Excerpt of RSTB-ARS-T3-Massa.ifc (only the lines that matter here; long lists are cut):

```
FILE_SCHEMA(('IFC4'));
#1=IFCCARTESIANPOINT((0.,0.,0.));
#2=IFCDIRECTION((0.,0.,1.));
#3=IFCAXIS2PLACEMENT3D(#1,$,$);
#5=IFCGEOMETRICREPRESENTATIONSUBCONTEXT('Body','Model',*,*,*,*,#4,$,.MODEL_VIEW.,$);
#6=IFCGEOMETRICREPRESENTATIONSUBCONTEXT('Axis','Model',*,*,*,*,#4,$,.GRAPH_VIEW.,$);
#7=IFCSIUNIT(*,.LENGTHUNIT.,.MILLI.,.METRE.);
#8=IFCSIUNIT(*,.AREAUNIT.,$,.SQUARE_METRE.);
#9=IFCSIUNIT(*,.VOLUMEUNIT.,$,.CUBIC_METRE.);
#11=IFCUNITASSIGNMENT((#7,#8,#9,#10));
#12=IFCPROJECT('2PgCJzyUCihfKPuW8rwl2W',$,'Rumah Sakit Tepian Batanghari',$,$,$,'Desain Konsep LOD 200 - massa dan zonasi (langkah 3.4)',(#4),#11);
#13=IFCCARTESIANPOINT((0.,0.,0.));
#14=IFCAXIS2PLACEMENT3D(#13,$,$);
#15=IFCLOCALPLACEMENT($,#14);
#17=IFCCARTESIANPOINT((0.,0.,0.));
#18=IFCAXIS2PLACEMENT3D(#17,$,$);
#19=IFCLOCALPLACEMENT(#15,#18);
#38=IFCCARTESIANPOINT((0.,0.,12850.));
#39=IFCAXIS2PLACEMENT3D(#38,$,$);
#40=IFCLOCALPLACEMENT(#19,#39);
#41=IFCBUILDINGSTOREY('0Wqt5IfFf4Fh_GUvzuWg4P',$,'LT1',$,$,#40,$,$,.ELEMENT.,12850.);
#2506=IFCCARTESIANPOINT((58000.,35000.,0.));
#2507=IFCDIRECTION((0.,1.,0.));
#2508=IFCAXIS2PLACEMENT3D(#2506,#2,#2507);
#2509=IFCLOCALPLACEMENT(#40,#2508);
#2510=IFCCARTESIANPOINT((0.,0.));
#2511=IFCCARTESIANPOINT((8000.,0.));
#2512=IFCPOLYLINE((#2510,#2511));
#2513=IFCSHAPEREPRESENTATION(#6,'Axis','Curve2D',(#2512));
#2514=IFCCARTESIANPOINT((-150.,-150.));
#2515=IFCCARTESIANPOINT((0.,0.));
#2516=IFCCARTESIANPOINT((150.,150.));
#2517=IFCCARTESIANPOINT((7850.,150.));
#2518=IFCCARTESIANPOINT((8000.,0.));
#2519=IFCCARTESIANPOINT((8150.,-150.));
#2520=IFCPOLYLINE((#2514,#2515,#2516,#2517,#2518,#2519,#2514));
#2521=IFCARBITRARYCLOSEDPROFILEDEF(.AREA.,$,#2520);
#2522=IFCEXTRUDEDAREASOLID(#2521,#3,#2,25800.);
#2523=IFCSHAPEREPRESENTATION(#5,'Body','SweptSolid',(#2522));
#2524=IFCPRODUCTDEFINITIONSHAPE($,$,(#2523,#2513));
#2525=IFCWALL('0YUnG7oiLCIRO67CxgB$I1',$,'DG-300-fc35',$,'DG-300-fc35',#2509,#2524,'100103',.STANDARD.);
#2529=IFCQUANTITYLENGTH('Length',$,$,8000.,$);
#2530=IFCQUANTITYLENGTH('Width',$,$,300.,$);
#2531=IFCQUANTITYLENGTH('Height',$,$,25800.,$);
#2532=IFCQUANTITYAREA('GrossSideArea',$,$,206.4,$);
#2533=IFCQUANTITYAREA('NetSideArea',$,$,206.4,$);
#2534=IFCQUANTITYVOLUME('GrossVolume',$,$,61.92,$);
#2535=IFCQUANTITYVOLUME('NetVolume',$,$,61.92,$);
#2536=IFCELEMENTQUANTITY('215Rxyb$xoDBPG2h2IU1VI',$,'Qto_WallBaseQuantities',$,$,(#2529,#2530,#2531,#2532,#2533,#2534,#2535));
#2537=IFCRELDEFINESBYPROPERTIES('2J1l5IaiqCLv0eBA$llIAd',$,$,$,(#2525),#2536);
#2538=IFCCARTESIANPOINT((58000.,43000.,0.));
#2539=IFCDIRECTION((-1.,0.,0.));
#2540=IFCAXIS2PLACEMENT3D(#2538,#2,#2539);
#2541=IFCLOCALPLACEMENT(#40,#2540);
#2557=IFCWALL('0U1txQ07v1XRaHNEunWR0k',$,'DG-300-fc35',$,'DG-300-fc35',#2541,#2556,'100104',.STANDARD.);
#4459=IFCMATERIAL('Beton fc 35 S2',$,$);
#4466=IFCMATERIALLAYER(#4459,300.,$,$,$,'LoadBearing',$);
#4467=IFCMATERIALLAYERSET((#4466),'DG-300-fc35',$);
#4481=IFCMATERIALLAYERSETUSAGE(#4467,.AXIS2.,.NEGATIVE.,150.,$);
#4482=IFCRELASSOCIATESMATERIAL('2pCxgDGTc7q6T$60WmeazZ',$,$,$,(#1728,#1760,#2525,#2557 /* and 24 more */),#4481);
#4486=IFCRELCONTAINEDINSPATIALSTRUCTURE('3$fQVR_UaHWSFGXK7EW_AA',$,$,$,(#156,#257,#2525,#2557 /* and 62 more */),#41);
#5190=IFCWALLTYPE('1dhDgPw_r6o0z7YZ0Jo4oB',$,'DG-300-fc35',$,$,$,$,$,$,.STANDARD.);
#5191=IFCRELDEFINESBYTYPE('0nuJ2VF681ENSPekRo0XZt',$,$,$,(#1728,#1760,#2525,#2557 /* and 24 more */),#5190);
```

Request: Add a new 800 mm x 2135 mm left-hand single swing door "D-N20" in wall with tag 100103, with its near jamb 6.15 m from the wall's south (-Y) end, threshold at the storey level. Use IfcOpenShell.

```python
import numpy as np
import ifcopenshell
import ifcopenshell.api.feature
import ifcopenshell.api.geometry
import ifcopenshell.api.pset
import ifcopenshell.api.root
import ifcopenshell.api.spatial
import ifcopenshell.geom
import ifcopenshell.util.element
import ifcopenshell.util.placement
import ifcopenshell.util.representation
import ifcopenshell.util.shape
import ifcopenshell.util.unit

model = ifcopenshell.open("RSTB-ARS-T3-Massa.ifc")
unit_scale = ifcopenshell.util.unit.calculate_unit_scale(model)
area_scale = ifcopenshell.util.unit.calculate_unit_scale(model, "AREAUNIT")
volume_scale = ifcopenshell.util.unit.calculate_unit_scale(model, "VOLUMEUNIT")
settings = ifcopenshell.geom.settings()


def volume(element):
    """Net volume in cubic metres, openings subtracted."""
    shape = ifcopenshell.geom.create_shape(settings, element)
    return ifcopenshell.util.shape.get_volume(shape.geometry)


wall = model.by_guid("0YUnG7oiLCIRO67CxgB$I1")
storey = ifcopenshell.util.element.get_container(wall, ifc_class="IfcBuildingStorey")
context = ifcopenshell.util.representation.get_context(model, "Model", "Body", "MODEL_VIEW")
before = volume(wall)

width, height, from_end, sill = 0.8, 2.135, 6.15, 0.0  # metres

# The wall runs along its own X axis, and the end named is its -X end.
wall_shape = ifcopenshell.geom.create_shape(settings, wall)
x, y, z = ifcopenshell.util.shape.get_vertices(wall_shape.geometry).T
start = x.min() + from_end
face, thickness = float(y.min()), float(y.max() - y.min())
wall_matrix = ifcopenshell.util.placement.get_local_placement(wall.ObjectPlacement)
level = ifcopenshell.util.placement.get_local_placement(storey.ObjectPlacement)[2, 3]


def in_wall(x, y):
    """Placement at x, y metres in the wall's axes, at sill height."""
    matrix = wall_matrix.copy()
    matrix[:, 3] = wall_matrix @ np.array([x / unit_scale, y / unit_scale, 0.0, 1.0])
    matrix[2, 3] = level + sill / unit_scale
    return matrix


# Opening: a box that overshoots both wall faces by 50 mm.
opening = ifcopenshell.api.root.create_entity(model, ifc_class="IfcOpeningElement", predefined_type="OPENING")
box = ifcopenshell.api.geometry.add_wall_representation(
    model, context=context, length=width, height=height, thickness=thickness + 0.1
)
ifcopenshell.api.geometry.assign_representation(model, product=opening, representation=box)
ifcopenshell.api.geometry.edit_object_placement(model, product=opening, matrix=in_wall(start, face - 0.05), is_si=False)
ifcopenshell.api.feature.add_feature(model, feature=opening, element=wall)

door = ifcopenshell.api.root.create_entity(model, ifc_class="IfcDoor", name="D-N20", predefined_type="DOOR")
door.OverallWidth, door.OverallHeight = width / unit_scale, height / unit_scale
door.OperationType = "SINGLE_SWING_LEFT"
body = ifcopenshell.api.geometry.add_door_representation(
    model,
    context=context,
    overall_width=door.OverallWidth,
    overall_height=door.OverallHeight,
    operation_type="SINGLE_SWING_LEFT",
    lining_properties={"LiningDepth": thickness / unit_scale, "ThresholdDepth": thickness / unit_scale},
)
ifcopenshell.api.geometry.assign_representation(model, product=door, representation=body)
ifcopenshell.api.spatial.assign_container(model, products=[door], relating_structure=storey)
ifcopenshell.api.feature.add_filling(model, opening=opening, element=door)

# The lining spans the wall, so the door starts at the wall face.
ifcopenshell.api.geometry.edit_object_placement(model, product=door, matrix=in_wall(start, face), is_si=False)

after = volume(wall)

# Update the wall's stored quantities.
qto = model.by_id(ifcopenshell.util.element.get_pset(wall, "Qto_WallBaseQuantities", should_inherit=False)["id"])
ifcopenshell.api.pset.edit_qto(model, qto=qto, properties={
    "NetSideArea": after / thickness / area_scale,
    "NetVolume": after / volume_scale,
})

print(f"wall volume {before:.3f} -> {after:.3f} m3")

model.write("RSTB-ARS-T3-Massa_v2.ifc")
```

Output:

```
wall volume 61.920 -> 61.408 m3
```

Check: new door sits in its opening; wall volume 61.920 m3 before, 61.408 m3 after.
